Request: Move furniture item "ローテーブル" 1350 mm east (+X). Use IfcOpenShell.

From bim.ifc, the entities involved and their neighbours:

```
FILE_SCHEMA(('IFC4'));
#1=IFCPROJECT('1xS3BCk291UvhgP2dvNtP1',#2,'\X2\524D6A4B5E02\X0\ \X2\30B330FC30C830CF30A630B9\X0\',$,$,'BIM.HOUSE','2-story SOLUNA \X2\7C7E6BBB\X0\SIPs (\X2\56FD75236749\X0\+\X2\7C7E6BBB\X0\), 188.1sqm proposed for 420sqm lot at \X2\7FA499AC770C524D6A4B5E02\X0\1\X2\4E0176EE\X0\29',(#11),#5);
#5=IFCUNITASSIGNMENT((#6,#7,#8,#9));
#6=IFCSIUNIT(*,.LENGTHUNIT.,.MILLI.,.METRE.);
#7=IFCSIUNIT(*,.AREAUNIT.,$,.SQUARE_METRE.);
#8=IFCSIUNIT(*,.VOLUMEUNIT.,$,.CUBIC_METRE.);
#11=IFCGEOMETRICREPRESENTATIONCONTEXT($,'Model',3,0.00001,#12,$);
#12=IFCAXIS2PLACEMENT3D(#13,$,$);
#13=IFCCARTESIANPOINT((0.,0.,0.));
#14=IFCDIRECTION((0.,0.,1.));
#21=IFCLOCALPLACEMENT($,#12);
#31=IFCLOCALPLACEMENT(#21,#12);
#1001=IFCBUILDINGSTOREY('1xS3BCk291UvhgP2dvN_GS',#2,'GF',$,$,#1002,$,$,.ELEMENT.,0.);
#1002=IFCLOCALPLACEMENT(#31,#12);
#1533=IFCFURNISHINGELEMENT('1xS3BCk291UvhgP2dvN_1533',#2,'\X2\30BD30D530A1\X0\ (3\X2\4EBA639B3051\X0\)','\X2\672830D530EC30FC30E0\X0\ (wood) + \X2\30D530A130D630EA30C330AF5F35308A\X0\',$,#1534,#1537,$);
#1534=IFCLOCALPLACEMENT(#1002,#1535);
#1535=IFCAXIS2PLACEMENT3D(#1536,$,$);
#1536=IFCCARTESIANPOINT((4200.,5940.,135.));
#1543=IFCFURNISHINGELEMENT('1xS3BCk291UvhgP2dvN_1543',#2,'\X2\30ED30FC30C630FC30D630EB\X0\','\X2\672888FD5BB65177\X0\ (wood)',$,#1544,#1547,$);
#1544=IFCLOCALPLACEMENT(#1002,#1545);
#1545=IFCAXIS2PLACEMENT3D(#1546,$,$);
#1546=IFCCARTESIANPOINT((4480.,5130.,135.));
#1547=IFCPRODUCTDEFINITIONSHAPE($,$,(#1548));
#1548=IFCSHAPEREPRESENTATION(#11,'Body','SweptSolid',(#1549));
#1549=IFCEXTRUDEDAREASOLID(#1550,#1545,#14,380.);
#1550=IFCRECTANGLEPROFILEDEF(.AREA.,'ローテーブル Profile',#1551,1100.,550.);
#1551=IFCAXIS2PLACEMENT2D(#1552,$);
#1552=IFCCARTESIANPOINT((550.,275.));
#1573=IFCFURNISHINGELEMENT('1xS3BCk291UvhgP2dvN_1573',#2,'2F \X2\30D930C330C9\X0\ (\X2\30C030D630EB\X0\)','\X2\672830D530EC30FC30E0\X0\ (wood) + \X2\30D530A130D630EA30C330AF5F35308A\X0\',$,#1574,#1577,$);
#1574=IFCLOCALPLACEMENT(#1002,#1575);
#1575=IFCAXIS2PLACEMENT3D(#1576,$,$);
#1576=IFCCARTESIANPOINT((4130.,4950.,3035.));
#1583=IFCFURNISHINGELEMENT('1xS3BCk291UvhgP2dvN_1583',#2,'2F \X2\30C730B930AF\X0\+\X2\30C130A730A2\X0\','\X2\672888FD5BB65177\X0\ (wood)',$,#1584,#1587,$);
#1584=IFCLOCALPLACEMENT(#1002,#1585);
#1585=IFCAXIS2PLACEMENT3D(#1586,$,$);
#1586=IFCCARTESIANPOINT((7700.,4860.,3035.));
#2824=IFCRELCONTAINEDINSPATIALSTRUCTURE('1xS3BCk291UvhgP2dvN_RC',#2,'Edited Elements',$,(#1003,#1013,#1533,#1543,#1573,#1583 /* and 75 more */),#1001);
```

```python
import ifcopenshell
import ifcopenshell.api.geometry
import ifcopenshell.util.placement

model = ifcopenshell.open("bim.ifc")

item = model.by_guid("1xS3BCk291UvhgP2dvN_1543")
matrix = ifcopenshell.util.placement.get_local_placement(item.ObjectPlacement)
matrix[0, 3] += 1350.0
ifcopenshell.api.geometry.edit_object_placement(model, product=item, matrix=matrix, is_si=False)

print(ifcopenshell.util.placement.get_local_placement(item.ObjectPlacement).round(3) + 0.0)

model.write("bim_v2.ifc")
```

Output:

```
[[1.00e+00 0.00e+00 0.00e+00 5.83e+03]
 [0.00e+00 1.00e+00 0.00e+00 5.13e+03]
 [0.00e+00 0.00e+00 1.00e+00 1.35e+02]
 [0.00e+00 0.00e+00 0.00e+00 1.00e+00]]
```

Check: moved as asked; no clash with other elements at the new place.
